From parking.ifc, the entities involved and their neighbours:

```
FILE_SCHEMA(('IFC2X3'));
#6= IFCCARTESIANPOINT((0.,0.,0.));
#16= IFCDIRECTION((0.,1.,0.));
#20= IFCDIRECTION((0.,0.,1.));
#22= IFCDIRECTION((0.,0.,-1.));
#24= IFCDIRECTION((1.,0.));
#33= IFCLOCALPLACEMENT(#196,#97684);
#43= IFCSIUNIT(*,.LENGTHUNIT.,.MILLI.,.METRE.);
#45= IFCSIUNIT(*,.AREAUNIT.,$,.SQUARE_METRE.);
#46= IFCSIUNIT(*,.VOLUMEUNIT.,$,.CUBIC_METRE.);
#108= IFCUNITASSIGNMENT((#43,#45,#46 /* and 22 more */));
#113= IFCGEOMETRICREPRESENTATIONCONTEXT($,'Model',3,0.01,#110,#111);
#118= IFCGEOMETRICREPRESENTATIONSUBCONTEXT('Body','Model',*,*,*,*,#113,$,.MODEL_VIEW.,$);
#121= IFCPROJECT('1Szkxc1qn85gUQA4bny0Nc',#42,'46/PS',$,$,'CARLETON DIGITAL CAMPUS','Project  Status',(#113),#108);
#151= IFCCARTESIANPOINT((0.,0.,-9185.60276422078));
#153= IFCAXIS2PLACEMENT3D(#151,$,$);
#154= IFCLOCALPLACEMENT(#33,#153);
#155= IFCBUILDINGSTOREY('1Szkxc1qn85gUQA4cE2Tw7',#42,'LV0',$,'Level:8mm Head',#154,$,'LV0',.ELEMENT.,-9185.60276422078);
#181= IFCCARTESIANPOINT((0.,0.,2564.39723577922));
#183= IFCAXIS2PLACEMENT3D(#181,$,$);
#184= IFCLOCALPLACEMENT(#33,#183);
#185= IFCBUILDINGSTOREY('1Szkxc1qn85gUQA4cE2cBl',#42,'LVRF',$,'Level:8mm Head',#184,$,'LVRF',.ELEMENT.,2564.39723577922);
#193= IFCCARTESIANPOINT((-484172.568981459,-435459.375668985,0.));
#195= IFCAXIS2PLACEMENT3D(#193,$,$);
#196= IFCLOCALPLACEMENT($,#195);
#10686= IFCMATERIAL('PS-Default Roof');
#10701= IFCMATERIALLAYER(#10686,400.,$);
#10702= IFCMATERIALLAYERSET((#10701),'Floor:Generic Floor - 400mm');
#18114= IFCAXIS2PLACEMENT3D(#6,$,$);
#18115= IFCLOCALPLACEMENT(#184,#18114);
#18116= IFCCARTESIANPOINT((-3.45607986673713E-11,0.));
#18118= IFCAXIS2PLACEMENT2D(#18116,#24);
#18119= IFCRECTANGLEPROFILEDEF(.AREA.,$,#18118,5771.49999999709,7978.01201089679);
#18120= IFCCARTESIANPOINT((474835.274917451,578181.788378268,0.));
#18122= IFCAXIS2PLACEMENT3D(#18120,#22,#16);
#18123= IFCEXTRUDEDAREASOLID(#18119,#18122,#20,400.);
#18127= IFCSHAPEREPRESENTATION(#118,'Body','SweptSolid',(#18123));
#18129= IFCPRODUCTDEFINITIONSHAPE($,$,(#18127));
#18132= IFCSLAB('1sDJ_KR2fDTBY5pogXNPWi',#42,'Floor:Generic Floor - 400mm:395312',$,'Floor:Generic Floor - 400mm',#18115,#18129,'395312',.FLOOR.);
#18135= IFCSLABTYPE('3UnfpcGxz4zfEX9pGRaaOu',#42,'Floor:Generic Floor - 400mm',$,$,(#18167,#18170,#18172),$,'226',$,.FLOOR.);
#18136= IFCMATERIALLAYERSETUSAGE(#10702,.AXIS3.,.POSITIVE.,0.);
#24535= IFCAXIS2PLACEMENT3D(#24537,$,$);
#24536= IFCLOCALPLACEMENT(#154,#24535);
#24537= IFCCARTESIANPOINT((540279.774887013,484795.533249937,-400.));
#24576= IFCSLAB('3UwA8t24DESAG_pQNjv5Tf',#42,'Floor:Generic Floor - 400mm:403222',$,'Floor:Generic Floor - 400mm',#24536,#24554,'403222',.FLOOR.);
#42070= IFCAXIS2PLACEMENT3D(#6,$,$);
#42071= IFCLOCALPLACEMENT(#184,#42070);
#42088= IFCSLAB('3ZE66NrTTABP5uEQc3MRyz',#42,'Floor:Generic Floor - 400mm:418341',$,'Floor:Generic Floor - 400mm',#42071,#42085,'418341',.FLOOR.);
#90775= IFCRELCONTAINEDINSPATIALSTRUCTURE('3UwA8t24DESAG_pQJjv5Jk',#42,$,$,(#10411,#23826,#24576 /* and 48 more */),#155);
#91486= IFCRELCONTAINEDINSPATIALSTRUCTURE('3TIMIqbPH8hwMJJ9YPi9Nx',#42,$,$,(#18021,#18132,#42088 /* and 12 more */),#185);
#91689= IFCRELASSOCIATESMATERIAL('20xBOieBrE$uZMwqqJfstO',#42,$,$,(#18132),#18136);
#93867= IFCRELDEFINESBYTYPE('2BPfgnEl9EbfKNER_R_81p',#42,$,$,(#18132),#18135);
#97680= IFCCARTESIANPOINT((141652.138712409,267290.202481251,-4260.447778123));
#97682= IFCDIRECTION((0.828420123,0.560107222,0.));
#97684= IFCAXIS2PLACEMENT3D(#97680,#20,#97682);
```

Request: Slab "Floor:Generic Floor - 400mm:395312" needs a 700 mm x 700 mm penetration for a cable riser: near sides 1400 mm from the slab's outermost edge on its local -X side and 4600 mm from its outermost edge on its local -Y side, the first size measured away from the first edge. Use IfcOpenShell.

```python
import numpy as np
import ifcopenshell
import ifcopenshell.api.feature
import ifcopenshell.api.geometry
import ifcopenshell.api.root
import ifcopenshell.geom
import ifcopenshell.util.placement
import ifcopenshell.util.representation
import ifcopenshell.util.shape
import ifcopenshell.util.unit

model = ifcopenshell.open("parking.ifc")
unit_scale = ifcopenshell.util.unit.calculate_unit_scale(model)
settings = ifcopenshell.geom.settings()


def volume(element):
    """Net volume in cubic metres, openings subtracted."""
    shape = ifcopenshell.geom.create_shape(settings, element)
    return ifcopenshell.util.shape.get_volume(shape.geometry)


slab = model.by_guid("1sDJ_KR2fDTBY5pogXNPWi")
before = volume(slab)

# Extent in the slab's own axes, in metres. The edges named are its -X and -Y sides.
slab_shape = ifcopenshell.geom.create_shape(settings, slab)
vertices = ifcopenshell.util.shape.get_vertices(slab_shape.geometry)
x_min, y_min, bottom = vertices.min(axis=0)
top = vertices[:, 2].max()

opening = ifcopenshell.api.root.create_entity(model, ifc_class="IfcOpeningElement", name="Cable riser opening")
context = ifcopenshell.util.representation.get_context(model, "Model", "Body", "MODEL_VIEW")
width, depth = 0.7, 0.7
outline = [(0.0, 0.0), (width, 0.0), (width, depth), (0.0, depth), (0.0, 0.0)]
# Overshoot both faces by 50 mm so the cut is clean.
shape = ifcopenshell.api.geometry.add_slab_representation(
    model, context=context, depth=top - bottom + 0.1, polyline=outline
)
ifcopenshell.api.geometry.assign_representation(model, product=opening, representation=shape)

matrix = ifcopenshell.util.placement.get_local_placement(slab.ObjectPlacement)
matrix[:, 3] = matrix @ np.append(np.array([x_min + 1.4, y_min + 4.6, bottom - 0.05]) / unit_scale, 1.0)
ifcopenshell.api.geometry.edit_object_placement(model, product=opening, matrix=matrix, is_si=False)
ifcopenshell.api.feature.add_feature(model, feature=opening, element=slab)

after = volume(slab)

print(f"slab volume {before:.3f} -> {after:.3f} m3")

model.write("parking-out.ifc")
```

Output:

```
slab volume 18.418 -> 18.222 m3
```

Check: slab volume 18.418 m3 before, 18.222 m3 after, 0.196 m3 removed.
